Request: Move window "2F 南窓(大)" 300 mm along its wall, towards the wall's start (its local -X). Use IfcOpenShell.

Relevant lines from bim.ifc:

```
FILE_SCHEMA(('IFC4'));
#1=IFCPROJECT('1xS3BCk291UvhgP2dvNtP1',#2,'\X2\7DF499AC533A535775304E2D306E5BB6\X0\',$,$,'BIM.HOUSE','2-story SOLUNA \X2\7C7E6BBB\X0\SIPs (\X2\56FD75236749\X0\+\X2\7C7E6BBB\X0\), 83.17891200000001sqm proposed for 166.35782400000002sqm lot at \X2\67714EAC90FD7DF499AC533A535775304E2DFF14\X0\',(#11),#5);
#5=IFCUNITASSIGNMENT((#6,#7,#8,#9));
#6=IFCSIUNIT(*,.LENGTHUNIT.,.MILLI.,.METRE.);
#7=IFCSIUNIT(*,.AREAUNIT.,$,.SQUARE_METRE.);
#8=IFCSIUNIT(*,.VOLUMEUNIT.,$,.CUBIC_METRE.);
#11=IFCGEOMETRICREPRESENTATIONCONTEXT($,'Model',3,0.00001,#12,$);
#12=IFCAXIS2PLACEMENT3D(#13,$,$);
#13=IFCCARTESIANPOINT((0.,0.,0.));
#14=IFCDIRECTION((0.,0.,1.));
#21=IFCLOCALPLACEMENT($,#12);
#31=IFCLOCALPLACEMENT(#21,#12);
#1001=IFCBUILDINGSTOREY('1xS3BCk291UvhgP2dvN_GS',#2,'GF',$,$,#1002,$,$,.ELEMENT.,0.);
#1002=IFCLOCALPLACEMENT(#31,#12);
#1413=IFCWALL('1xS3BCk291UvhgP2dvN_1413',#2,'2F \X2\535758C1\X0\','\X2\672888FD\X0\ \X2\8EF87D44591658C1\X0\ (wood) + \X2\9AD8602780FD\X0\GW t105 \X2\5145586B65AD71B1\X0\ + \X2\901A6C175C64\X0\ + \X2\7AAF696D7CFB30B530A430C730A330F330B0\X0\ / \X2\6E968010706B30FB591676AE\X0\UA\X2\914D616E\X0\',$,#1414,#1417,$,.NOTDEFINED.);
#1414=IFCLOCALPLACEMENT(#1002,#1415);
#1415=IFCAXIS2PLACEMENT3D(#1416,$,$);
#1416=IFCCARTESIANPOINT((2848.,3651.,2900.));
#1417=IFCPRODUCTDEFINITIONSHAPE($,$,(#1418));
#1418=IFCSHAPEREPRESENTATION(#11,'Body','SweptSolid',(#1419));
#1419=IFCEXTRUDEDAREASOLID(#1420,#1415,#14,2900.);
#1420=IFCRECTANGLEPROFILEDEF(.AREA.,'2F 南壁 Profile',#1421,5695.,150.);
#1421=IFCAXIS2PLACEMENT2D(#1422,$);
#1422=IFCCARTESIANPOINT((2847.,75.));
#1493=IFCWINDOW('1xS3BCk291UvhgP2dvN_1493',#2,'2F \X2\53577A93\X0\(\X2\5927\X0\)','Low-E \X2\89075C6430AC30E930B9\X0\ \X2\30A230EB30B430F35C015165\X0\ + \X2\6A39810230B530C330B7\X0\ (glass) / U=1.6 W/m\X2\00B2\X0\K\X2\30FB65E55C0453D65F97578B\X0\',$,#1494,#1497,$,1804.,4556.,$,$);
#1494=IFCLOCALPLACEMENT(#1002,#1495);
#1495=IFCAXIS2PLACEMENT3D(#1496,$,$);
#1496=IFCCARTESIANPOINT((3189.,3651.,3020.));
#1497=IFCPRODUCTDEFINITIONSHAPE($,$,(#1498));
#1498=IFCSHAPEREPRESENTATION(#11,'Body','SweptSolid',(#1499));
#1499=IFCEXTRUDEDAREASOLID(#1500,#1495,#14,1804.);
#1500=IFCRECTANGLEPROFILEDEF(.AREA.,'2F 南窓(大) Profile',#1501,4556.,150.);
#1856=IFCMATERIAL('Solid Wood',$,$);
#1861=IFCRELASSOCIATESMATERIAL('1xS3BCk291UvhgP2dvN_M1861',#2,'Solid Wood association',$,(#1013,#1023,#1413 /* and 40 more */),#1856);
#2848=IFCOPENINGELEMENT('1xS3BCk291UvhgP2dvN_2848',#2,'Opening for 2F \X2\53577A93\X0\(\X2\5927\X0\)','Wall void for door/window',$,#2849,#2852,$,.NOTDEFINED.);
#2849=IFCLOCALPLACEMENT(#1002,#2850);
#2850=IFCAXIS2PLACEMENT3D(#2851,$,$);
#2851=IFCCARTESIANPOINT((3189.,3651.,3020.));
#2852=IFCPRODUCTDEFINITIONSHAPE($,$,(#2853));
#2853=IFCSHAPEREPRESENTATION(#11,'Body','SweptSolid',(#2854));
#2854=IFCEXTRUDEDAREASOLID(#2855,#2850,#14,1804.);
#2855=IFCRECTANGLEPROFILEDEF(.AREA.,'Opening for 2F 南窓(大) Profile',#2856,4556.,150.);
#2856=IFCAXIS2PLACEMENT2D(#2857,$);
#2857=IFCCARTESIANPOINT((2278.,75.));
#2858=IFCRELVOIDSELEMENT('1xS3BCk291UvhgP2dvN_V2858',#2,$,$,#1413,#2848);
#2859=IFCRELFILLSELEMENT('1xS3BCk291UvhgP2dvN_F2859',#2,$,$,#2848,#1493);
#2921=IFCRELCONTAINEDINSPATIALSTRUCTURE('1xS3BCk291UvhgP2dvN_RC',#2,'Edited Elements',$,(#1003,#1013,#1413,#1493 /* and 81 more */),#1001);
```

```python
import ifcopenshell
import ifcopenshell.api.geometry
import ifcopenshell.util.placement
import ifcopenshell.util.unit

model = ifcopenshell.open("bim.ifc")
unit_scale = ifcopenshell.util.unit.calculate_unit_scale(model)

window = model.by_id(1493)
opening = window.FillsVoids[0].RelatingOpeningElement
wall = opening.VoidsElements[0].RelatingBuildingElement

wall_matrix = ifcopenshell.util.placement.get_local_placement(wall.ObjectPlacement)
shift = wall_matrix[:3, 0] * -0.3 / unit_scale
before = ifcopenshell.util.placement.get_local_placement(window.ObjectPlacement)[:3, 3].copy()

# The window is not placed relative to its opening, so move both.
for product in (opening, window):
    matrix = ifcopenshell.util.placement.get_local_placement(product.ObjectPlacement)
    matrix[:3, 3] += shift
    ifcopenshell.api.geometry.edit_object_placement(model, product=product, matrix=matrix, is_si=False)

after = ifcopenshell.util.placement.get_local_placement(window.ObjectPlacement)[:3, 3]
print("window moved by", (after - before).round(3) + 0.0)

model.write("bim-out.ifc")
```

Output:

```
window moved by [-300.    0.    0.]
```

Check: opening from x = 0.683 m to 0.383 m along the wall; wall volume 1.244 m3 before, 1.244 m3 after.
